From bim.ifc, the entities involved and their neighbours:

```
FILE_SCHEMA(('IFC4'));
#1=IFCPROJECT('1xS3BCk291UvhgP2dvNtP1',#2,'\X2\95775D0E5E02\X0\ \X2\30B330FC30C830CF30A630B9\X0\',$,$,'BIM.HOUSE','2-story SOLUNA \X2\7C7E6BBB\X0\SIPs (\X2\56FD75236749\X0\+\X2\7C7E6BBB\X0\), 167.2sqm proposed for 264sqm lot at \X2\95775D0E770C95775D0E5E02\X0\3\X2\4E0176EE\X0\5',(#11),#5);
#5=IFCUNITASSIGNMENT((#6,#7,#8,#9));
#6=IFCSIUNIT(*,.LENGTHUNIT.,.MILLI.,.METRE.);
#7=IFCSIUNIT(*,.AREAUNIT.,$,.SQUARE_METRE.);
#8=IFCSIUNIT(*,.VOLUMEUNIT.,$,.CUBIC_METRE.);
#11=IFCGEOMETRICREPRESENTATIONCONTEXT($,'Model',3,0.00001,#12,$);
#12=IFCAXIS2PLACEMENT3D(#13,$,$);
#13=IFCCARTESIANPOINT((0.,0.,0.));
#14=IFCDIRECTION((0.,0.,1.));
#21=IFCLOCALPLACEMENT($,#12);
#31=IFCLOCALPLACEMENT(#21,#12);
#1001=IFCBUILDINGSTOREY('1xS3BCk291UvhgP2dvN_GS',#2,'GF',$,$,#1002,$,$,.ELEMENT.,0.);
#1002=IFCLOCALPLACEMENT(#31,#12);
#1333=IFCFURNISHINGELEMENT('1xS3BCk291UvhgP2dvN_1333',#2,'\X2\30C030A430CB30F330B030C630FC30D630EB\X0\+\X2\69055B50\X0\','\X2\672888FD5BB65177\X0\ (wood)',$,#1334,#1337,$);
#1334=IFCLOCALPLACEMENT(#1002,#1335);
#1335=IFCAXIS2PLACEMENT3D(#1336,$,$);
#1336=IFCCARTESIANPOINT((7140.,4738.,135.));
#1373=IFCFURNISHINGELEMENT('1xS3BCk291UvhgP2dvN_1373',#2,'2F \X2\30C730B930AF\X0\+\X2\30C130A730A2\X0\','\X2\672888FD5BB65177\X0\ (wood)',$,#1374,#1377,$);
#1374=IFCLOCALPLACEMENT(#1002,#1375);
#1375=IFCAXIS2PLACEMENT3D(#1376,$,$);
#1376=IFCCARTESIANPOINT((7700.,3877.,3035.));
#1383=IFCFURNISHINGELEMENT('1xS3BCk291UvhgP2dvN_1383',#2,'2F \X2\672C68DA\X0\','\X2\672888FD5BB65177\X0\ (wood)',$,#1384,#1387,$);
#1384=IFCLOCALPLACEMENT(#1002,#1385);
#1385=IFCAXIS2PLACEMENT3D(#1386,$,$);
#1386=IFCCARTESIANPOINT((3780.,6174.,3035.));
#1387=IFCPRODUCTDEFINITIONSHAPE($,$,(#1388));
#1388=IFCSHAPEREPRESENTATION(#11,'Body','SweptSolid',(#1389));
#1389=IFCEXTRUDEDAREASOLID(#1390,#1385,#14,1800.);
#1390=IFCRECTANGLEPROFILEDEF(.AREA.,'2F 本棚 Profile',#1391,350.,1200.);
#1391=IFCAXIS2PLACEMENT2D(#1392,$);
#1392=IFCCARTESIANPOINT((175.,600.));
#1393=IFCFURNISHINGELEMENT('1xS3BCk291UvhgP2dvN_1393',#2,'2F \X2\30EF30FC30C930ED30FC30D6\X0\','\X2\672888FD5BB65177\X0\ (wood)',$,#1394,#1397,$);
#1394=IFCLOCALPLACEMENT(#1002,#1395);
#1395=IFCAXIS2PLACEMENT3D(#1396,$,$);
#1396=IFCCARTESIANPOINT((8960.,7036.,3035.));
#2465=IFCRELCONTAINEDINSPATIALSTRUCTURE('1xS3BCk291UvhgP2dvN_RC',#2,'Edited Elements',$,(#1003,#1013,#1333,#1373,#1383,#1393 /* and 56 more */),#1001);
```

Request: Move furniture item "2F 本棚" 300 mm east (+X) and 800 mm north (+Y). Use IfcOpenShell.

```python
import ifcopenshell
import ifcopenshell.api.geometry
import ifcopenshell.util.placement
import ifcopenshell.util.unit

model = ifcopenshell.open("bim.ifc")
unit_scale = ifcopenshell.util.unit.calculate_unit_scale(model)

item = model.by_guid("1xS3BCk291UvhgP2dvN_1383")
matrix = ifcopenshell.util.placement.get_local_placement(item.ObjectPlacement)
matrix[0, 3] += 0.3 / unit_scale
matrix[1, 3] += 0.8 / unit_scale
ifcopenshell.api.geometry.edit_object_placement(model, product=item, matrix=matrix, is_si=False)

print(ifcopenshell.util.placement.get_local_placement(item.ObjectPlacement).round(3) + 0.0)

model.write("bim_v2.ifc")
```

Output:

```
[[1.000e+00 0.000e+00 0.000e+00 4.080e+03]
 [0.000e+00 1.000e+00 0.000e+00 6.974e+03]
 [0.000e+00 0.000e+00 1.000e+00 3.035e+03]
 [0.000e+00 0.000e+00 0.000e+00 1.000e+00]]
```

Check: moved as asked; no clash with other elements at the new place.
